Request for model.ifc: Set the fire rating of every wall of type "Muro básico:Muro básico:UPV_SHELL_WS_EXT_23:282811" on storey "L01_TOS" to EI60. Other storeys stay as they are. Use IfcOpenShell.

First a look at what the model holds.

```python
import ifcopenshell
import ifcopenshell.util.element

model = ifcopenshell.open("model.ifc")
print(model.schema)
storey = next(s for s in model.by_type("IfcBuildingStorey") if s.Name == "L01_TOS")
walls = [e for e in ifcopenshell.util.element.get_decomposition(storey) if e.is_a("IfcWall")]
seen = {}
for e in walls:
    element_type = ifcopenshell.util.element.get_type(e)
    key = (element_type.Name if element_type != e and element_type else None, ifcopenshell.util.element.get_pset(e, "Pset_WallCommon", "FireRating"))
    seen[key] = seen.get(key, 0) + 1
for (name, value), count in sorted(seen.items(), key=str):
    print(count, "x", name, "|", value)
```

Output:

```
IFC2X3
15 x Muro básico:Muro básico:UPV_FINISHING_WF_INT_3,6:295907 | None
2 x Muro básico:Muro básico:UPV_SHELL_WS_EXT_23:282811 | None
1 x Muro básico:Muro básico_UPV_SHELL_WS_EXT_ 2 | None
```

```python
import ifcopenshell
import ifcopenshell.api.pset
import ifcopenshell.util.element

model = ifcopenshell.open("model.ifc")

storey = next(s for s in model.by_type("IfcBuildingStorey") if s.Name == "L01_TOS")
walls = [e for e in ifcopenshell.util.element.get_decomposition(storey) if e.is_a("IfcWall")]

count = 0
for e in walls:
    element_type = ifcopenshell.util.element.get_type(e)
    if element_type in (None, e) or element_type.Name != "Muro básico:Muro básico:UPV_SHELL_WS_EXT_23:282811":
        continue
    # add_pset returns the element's existing set when there is one.
    pset = ifcopenshell.api.pset.add_pset(model, product=e, name="Pset_WallCommon")
    ifcopenshell.api.pset.edit_pset(model, pset=pset, properties={"FireRating": "EI60"})
    count += 1

print(count, "walls updated")

model.write("model_v2.ifc")
```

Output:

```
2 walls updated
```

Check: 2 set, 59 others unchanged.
